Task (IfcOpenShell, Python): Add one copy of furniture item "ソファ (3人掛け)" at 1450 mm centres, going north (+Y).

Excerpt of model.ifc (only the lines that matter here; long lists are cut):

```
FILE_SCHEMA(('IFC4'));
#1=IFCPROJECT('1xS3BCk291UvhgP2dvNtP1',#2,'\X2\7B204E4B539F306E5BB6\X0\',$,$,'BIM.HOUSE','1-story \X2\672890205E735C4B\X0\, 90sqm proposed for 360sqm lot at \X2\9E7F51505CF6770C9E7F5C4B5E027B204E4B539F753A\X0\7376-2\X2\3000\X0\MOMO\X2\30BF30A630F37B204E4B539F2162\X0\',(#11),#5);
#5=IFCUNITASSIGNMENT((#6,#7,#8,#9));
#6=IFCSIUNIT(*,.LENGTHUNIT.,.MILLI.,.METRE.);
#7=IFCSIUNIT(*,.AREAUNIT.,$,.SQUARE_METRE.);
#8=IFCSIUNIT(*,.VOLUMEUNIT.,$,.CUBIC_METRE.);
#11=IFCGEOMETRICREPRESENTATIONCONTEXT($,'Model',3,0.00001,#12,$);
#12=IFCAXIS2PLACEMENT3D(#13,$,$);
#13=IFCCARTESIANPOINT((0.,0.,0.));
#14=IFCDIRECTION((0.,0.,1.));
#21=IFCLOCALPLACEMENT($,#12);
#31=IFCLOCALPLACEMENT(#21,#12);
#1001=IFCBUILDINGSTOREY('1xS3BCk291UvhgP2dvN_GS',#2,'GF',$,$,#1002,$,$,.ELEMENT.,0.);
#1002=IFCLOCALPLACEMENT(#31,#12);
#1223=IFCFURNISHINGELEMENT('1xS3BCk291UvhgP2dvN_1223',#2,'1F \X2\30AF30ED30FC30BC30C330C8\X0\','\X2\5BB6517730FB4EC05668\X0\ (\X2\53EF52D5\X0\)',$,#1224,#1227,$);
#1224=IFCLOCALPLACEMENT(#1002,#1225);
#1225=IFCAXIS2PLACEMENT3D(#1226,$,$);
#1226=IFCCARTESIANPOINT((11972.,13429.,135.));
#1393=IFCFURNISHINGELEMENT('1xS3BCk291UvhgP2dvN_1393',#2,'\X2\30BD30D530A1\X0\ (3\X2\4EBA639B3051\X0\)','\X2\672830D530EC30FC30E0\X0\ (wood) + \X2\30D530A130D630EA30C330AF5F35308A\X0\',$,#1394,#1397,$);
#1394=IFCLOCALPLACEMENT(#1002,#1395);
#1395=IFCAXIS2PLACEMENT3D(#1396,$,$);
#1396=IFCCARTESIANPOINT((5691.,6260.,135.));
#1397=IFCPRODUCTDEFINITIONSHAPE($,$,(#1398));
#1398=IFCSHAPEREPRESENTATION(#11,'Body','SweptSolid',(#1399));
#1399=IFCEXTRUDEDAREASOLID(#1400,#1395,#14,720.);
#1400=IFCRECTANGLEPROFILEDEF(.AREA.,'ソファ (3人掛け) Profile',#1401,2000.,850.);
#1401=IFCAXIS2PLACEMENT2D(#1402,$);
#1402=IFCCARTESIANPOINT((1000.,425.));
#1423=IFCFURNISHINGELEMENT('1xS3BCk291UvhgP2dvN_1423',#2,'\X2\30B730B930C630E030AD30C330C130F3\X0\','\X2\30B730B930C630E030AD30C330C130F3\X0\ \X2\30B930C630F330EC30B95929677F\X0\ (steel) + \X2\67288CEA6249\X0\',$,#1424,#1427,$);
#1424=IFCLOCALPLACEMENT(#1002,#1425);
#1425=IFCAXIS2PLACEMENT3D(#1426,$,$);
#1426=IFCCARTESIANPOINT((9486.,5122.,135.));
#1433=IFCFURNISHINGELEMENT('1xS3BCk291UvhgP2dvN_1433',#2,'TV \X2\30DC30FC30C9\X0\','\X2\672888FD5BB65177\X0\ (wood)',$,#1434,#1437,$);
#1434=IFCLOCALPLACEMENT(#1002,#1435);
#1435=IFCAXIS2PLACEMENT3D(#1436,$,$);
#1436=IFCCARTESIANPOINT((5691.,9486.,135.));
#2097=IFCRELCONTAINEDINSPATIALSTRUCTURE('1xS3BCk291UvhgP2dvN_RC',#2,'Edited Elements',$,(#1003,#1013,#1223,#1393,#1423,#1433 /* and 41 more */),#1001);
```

```python
import numpy as np
import ifcopenshell
import ifcopenshell.api.geometry
import ifcopenshell.api.root
import ifcopenshell.util.element
import ifcopenshell.util.placement
import ifcopenshell.util.unit

model = ifcopenshell.open("model.ifc")
unit_scale = ifcopenshell.util.unit.calculate_unit_scale(model)


def reuse_history(source, copy):
    """copy_class also copies each property set's owner history, people and application; keep the originals."""
    for rel in copy.IsDefinedBy:
        if rel.is_a("IfcRelDefinesByProperties") and (history := rel.RelatingPropertyDefinition.OwnerHistory):
            rel.RelatingPropertyDefinition.OwnerHistory = source.OwnerHistory
            ifcopenshell.util.element.remove_deep2(model, history)


source = model.by_guid("1xS3BCk291UvhgP2dvN_1393")
base = ifcopenshell.util.placement.get_local_placement(source.ObjectPlacement)
step = np.array([0.0, 1.0, 0.0]) * 1.45 / unit_scale

for i in range(1, 2):
    copy = ifcopenshell.api.root.copy_class(model, product=source)
    copy.Representation = ifcopenshell.util.element.copy_deep(
        model, source.Representation, exclude=["IfcGeometricRepresentationContext", "IfcRepresentationMap"]
    )
    reuse_history(source, copy)
    matrix = base.copy()
    matrix[:3, 3] += i * step
    print("added at", matrix[:3, 3].round(3) + 0.0)
    ifcopenshell.api.geometry.edit_object_placement(model, product=copy, matrix=matrix, is_si=False)

model.write("model_rev.ifc")
```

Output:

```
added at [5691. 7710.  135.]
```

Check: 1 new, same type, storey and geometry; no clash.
